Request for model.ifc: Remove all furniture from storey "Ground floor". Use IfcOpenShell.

First a look at what the model holds.

```python
import ifcopenshell
import ifcopenshell.util.element

model = ifcopenshell.open("model.ifc")
print(model.schema)
storey = next(s for s in model.by_type("IfcBuildingStorey") if s.Name == "Ground floor")
furniture = [e for e in ifcopenshell.util.element.get_decomposition(storey) if e.is_a("IfcFurnishingElement")]
seen = {}
for e in furniture:
    element_type = ifcopenshell.util.element.get_type(e)
    name = element_type.Name if element_type not in (None, e) else None
    seen[name] = seen.get(name, 0) + 1
for name, count in sorted(seen.items(), key=str):
    print(count, "x", name)
```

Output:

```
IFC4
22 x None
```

```python
import ifcopenshell
import ifcopenshell.api.root
import ifcopenshell.util.element

model = ifcopenshell.open("model.ifc")

storey = next(s for s in model.by_type("IfcBuildingStorey") if s.Name == "Ground floor")
furniture = [e for e in ifcopenshell.util.element.get_decomposition(storey) if e.is_a("IfcFurnishingElement")]

for e in furniture:
    ifcopenshell.api.root.remove_product(model, product=e)
print(len(furniture), "removed")

model.write("model_updated.ifc")
```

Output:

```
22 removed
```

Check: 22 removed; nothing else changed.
